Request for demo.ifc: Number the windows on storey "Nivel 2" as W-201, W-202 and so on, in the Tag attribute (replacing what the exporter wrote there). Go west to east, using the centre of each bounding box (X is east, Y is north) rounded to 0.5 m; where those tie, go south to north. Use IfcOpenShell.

First a look at what the model holds.

```python
import ifcopenshell
import ifcopenshell.util.element
import ifcopenshell.util.placement

model = ifcopenshell.open("demo.ifc")
print(model.schema)
storey = next(s for s in model.by_type("IfcBuildingStorey") if s.Name == "Nivel 2")
windows = [e for e in ifcopenshell.util.element.get_decomposition(storey) if e.is_a("IfcWindow")]
for e in sorted(windows, key=lambda e: e.id()):
    origin = ifcopenshell.util.placement.get_local_placement(e.ObjectPlacement)[:3, 3]
    print(e.id(), e.Tag, e.Name, origin.round(2) + 0.0, sep=" | ")
```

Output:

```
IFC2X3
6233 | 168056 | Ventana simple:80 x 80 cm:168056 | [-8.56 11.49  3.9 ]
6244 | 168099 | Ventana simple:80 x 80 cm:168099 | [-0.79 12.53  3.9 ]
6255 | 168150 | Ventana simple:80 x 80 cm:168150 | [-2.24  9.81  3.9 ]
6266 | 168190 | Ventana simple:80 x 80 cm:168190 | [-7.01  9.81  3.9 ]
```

```python
import ifcopenshell
import ifcopenshell.geom
import ifcopenshell.util.element
import ifcopenshell.util.shape

model = ifcopenshell.open("demo.ifc")
settings = ifcopenshell.geom.settings()
settings.set("use-world-coords", True)


def centre(element):
    shape = ifcopenshell.geom.create_shape(settings, element)
    return ifcopenshell.util.shape.get_bbox_centroid(shape.geometry)


storey = next(s for s in model.by_type("IfcBuildingStorey") if s.Name == "Nivel 2")
windows = [e for e in ifcopenshell.util.element.get_decomposition(storey) if e.is_a("IfcWindow")]

# Insertion points can sit at a corner or the storey origin, so sort by the geometry (in metres).
centres = {e: centre(e) for e in windows}
windows.sort(key=lambda e: (round(centres[e][0] / 0.5), centres[e][1]))

for i, e in enumerate(windows, start=1):
    number = f"W-2{i:02d}"
    e.Tag = number
    print(e.id(), number)

model.write("demo_edited.ifc")
```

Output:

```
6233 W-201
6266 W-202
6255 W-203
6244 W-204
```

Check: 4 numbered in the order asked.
